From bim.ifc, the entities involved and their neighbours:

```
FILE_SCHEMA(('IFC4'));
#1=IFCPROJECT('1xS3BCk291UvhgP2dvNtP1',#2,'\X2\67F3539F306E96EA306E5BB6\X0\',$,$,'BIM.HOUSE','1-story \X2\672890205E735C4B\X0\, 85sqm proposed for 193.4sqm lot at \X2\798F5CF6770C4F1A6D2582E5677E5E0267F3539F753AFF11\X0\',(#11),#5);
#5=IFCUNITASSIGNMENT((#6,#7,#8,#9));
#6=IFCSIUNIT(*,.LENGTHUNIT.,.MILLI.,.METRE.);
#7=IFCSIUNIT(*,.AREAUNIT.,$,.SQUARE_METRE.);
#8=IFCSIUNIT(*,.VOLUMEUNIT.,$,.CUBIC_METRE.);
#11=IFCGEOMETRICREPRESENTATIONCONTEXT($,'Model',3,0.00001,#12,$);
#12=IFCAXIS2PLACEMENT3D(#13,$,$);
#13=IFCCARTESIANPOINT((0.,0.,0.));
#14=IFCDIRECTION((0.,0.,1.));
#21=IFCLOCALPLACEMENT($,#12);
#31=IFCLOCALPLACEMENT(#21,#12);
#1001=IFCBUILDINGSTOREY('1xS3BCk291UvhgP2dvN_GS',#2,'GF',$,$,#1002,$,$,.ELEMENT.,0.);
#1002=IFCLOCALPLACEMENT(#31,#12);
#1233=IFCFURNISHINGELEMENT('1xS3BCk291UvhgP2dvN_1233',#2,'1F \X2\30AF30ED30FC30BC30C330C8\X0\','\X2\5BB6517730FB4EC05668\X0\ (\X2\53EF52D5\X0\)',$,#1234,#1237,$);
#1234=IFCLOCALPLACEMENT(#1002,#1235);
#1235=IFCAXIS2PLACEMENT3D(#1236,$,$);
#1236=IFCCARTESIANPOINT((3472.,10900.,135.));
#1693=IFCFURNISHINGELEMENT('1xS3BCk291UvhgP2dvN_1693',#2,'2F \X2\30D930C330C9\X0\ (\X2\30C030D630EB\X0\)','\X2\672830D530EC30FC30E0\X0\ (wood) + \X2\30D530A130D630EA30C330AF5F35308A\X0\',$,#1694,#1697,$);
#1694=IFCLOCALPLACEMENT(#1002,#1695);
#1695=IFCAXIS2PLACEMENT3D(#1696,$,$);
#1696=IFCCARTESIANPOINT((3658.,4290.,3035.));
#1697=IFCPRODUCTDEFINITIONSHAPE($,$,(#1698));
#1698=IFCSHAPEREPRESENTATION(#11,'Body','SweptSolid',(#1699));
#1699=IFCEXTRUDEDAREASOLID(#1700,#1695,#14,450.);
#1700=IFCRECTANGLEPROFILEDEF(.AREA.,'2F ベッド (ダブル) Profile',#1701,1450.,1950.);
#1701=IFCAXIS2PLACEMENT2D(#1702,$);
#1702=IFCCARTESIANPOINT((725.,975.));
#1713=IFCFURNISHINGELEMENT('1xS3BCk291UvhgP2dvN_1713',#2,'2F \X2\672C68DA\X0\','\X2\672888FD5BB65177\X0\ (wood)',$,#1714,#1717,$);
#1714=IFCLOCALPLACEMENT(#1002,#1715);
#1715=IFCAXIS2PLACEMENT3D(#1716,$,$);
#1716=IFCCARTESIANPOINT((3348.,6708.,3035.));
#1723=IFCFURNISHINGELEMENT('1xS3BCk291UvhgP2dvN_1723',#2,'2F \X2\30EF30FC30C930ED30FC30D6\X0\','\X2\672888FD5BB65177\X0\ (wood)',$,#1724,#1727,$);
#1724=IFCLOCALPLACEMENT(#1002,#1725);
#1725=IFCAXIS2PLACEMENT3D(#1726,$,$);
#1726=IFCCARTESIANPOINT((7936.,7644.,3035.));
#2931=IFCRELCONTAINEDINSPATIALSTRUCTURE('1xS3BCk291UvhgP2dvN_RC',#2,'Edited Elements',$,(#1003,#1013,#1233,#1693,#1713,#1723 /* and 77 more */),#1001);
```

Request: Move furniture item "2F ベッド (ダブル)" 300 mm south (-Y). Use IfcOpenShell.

```python
import ifcopenshell
import ifcopenshell.api.geometry
import ifcopenshell.util.placement
import ifcopenshell.util.unit

model = ifcopenshell.open("bim.ifc")
unit_scale = ifcopenshell.util.unit.calculate_unit_scale(model)

item = model.by_guid("1xS3BCk291UvhgP2dvN_1693")
matrix = ifcopenshell.util.placement.get_local_placement(item.ObjectPlacement)
matrix[1, 3] -= 0.3 / unit_scale
ifcopenshell.api.geometry.edit_object_placement(model, product=item, matrix=matrix, is_si=False)

print(ifcopenshell.util.placement.get_local_placement(item.ObjectPlacement).round(3) + 0.0)

model.write("bim_updated.ifc")
```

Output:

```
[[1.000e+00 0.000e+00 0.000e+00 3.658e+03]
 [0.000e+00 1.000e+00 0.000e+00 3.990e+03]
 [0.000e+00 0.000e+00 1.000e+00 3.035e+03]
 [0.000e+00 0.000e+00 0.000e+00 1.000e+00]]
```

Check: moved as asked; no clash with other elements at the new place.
